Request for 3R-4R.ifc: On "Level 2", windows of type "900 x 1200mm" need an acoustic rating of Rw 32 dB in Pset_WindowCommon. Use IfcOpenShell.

First a look at what the model holds.

```python
import ifcopenshell
import ifcopenshell.util.element

model = ifcopenshell.open("3R-4R.ifc")
print(model.schema)
storey = next(s for s in model.by_type("IfcBuildingStorey") if s.Name == "Level 2")
windows = [e for e in ifcopenshell.util.element.get_decomposition(storey) if e.is_a("IfcWindow")]
seen = {}
for e in windows:
    element_type = ifcopenshell.util.element.get_type(e)
    key = (element_type.Name if element_type != e and element_type else None, ifcopenshell.util.element.get_pset(e, "Pset_WindowCommon", "AcousticRating"))
    seen[key] = seen.get(key, 0) + 1
for (name, value), count in sorted(seen.items(), key=str):
    print(count, "x", name, "|", value)
```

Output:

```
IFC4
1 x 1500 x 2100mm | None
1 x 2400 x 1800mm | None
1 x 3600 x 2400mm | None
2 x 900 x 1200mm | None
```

```python
import ifcopenshell
import ifcopenshell.api.pset
import ifcopenshell.util.element

model = ifcopenshell.open("3R-4R.ifc")

storey = next(s for s in model.by_type("IfcBuildingStorey") if s.Name == "Level 2")
windows = [e for e in ifcopenshell.util.element.get_decomposition(storey) if e.is_a("IfcWindow")]

count = 0
for e in windows:
    element_type = ifcopenshell.util.element.get_type(e)
    if element_type in (None, e) or element_type.Name != "900 x 1200mm":
        continue
    # add_pset returns the element's existing set when there is one.
    pset = ifcopenshell.api.pset.add_pset(model, product=e, name="Pset_WindowCommon")
    ifcopenshell.api.pset.edit_pset(model, pset=pset, properties={"AcousticRating": "Rw 32 dB"})
    count += 1

print(count, "windows updated")

model.write("3R-4R_v2.ifc")
```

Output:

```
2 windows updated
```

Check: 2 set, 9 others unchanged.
